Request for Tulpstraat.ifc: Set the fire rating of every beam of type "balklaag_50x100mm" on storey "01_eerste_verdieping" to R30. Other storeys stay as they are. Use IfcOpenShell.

First a look at what the model holds.

```python
import ifcopenshell
import ifcopenshell.util.element

model = ifcopenshell.open("Tulpstraat.ifc")
print(model.schema)
storey = next(s for s in model.by_type("IfcBuildingStorey") if s.Name == "01_eerste_verdieping")
beams = [e for e in ifcopenshell.util.element.get_decomposition(storey) if e.is_a("IfcBeam")]
seen = {}
for e in beams:
    element_type = ifcopenshell.util.element.get_type(e)
    key = (element_type.Name if element_type != e and element_type else None, ifcopenshell.util.element.get_pset(e, "Pset_BeamCommon", "FireRating"))
    seen[key] = seen.get(key, 0) + 1
for (name, value), count in sorted(seen.items(), key=str):
    print(count, "x", name, "|", value)
```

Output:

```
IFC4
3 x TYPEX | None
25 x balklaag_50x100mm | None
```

```python
import ifcopenshell
import ifcopenshell.api.pset
import ifcopenshell.util.element

model = ifcopenshell.open("Tulpstraat.ifc")

storey = next(s for s in model.by_type("IfcBuildingStorey") if s.Name == "01_eerste_verdieping")
beams = [e for e in ifcopenshell.util.element.get_decomposition(storey) if e.is_a("IfcBeam")]

count = 0
for e in beams:
    element_type = ifcopenshell.util.element.get_type(e)
    if element_type in (None, e) or element_type.Name != "balklaag_50x100mm":
        continue
    # add_pset returns the element's existing set when there is one.
    pset = ifcopenshell.api.pset.add_pset(model, product=e, name="Pset_BeamCommon")
    ifcopenshell.api.pset.edit_pset(model, pset=pset, properties={"FireRating": "R30"})
    count += 1

print(count, "beams updated")

model.write("Tulpstraat_v2.ifc")
```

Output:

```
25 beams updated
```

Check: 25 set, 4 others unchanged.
